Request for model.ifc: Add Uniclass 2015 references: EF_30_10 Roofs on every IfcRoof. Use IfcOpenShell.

First a look at what the model holds.

```python
import ifcopenshell

model = ifcopenshell.open("model.ifc")
print(model.schema)
print("classifications:", [c.Name for c in model.by_type("IfcClassification")])
for ifc_class in ("IfcDoor", "IfcRoof", "IfcStair", "IfcWall", "IfcWindow"):
    print(ifc_class, len(model.by_type(ifc_class)))
```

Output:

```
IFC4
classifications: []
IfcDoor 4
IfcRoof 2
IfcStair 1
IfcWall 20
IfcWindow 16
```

```python
import ifcopenshell
import ifcopenshell.api.classification

model = ifcopenshell.open("model.ifc")

system = ifcopenshell.api.classification.add_classification(model, classification="Uniclass 2015")

codes = {
    "IfcRoof": ("EF_30_10", "Roofs"),
}
for ifc_class, (code, name) in codes.items():
    products = model.by_type(ifc_class)
    ifcopenshell.api.classification.add_reference(
        model, products=products, classification=system, identification=code, name=name
    )
    print(code, len(products))

model.write("model_rev.ifc")
```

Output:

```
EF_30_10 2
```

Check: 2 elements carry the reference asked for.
